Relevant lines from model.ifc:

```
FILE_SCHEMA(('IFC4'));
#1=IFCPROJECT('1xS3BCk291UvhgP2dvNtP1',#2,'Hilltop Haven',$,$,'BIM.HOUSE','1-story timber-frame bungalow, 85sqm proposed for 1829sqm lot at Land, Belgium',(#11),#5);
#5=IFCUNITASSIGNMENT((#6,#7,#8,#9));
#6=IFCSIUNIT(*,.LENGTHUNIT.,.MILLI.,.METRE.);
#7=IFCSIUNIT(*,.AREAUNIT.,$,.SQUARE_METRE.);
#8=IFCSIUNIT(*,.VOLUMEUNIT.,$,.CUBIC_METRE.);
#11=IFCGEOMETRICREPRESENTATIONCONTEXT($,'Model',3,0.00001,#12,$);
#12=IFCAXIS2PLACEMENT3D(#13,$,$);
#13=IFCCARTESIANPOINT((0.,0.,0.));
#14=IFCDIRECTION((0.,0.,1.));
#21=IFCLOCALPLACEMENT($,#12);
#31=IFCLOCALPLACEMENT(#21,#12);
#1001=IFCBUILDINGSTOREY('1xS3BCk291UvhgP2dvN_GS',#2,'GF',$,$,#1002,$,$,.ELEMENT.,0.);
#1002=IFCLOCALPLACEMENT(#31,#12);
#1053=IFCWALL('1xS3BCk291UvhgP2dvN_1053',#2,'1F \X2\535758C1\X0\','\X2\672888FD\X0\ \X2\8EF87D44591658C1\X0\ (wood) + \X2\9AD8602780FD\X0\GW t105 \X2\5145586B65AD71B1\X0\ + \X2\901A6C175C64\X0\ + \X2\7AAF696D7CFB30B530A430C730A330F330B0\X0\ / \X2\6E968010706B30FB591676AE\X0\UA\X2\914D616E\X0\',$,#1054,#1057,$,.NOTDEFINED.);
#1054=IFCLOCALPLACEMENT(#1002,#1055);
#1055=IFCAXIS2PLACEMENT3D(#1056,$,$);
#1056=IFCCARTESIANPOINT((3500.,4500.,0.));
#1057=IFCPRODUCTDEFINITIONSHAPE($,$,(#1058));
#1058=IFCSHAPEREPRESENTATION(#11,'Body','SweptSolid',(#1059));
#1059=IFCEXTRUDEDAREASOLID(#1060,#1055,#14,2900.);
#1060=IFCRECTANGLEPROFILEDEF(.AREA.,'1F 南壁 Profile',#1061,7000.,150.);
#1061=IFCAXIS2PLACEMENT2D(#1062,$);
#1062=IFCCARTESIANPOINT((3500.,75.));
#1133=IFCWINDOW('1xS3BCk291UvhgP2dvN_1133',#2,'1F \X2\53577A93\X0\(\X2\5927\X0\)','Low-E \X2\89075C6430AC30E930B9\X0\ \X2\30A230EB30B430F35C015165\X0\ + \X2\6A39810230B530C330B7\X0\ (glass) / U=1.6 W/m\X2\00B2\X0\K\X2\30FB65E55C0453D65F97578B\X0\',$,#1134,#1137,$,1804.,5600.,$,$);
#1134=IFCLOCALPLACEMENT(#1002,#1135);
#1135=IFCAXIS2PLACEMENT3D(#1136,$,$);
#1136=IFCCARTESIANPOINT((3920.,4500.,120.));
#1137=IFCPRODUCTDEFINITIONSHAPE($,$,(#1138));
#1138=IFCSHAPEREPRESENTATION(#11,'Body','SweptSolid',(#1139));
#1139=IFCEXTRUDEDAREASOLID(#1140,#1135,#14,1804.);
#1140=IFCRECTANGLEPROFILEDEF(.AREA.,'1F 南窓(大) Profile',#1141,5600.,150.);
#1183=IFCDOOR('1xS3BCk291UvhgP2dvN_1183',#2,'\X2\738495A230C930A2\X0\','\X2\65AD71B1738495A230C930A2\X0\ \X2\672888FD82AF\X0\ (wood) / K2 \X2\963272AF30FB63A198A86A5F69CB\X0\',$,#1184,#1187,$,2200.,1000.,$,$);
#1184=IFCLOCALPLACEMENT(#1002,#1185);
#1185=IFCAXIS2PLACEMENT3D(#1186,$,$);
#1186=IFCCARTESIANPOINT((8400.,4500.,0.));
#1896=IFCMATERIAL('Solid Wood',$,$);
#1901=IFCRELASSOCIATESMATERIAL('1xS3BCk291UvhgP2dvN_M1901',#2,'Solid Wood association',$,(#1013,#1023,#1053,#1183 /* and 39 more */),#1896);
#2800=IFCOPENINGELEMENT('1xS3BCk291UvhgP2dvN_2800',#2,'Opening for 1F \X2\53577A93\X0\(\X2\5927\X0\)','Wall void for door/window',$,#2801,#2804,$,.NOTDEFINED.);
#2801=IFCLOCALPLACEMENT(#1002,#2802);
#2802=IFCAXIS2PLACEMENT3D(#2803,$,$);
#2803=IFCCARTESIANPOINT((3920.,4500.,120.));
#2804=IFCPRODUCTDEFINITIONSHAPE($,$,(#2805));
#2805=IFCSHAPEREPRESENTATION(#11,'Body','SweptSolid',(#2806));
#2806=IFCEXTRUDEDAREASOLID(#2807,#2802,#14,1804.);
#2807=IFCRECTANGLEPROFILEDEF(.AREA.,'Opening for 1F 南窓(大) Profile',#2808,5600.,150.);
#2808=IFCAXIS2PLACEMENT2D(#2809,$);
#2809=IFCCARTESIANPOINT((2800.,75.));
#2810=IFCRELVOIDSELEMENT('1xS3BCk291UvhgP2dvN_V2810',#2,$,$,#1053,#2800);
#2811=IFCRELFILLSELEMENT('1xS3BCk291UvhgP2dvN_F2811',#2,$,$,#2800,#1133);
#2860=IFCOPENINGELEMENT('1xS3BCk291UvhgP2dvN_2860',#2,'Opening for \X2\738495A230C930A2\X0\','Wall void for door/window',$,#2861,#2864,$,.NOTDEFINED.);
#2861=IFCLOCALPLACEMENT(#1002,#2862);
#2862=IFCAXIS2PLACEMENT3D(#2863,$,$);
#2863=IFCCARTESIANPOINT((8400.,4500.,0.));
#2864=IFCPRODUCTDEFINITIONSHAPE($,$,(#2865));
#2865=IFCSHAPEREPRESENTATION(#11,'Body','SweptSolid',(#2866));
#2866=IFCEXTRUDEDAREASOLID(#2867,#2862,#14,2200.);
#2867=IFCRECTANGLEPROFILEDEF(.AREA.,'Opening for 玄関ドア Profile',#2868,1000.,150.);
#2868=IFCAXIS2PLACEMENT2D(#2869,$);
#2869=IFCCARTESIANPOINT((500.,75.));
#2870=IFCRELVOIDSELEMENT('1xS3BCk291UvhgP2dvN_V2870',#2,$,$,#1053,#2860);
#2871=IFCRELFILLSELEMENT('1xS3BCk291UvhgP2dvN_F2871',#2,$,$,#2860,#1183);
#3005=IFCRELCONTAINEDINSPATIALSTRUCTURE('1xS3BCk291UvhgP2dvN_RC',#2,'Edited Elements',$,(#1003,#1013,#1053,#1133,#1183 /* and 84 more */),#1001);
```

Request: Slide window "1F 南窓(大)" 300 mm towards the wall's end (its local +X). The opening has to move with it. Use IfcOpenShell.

```python
import ifcopenshell
import ifcopenshell.api.geometry
import ifcopenshell.util.placement

model = ifcopenshell.open("model.ifc")

window = model.by_guid("1xS3BCk291UvhgP2dvN_1133")
opening = window.FillsVoids[0].RelatingOpeningElement
wall = opening.VoidsElements[0].RelatingBuildingElement

wall_matrix = ifcopenshell.util.placement.get_local_placement(wall.ObjectPlacement)
shift = wall_matrix[:3, 0] * 300.0
before = ifcopenshell.util.placement.get_local_placement(window.ObjectPlacement)[:3, 3].copy()

# The window is not placed relative to its opening, so move both.
for product in (opening, window):
    matrix = ifcopenshell.util.placement.get_local_placement(product.ObjectPlacement)
    matrix[:3, 3] += shift
    ifcopenshell.api.geometry.edit_object_placement(model, product=product, matrix=matrix, is_si=False)

after = ifcopenshell.util.placement.get_local_placement(window.ObjectPlacement)[:3, 3]
print("window moved by", (after - before).round(3) + 0.0)

model.write("model_edited.ifc")
```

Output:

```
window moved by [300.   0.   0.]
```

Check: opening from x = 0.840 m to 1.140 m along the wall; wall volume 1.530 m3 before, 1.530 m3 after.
